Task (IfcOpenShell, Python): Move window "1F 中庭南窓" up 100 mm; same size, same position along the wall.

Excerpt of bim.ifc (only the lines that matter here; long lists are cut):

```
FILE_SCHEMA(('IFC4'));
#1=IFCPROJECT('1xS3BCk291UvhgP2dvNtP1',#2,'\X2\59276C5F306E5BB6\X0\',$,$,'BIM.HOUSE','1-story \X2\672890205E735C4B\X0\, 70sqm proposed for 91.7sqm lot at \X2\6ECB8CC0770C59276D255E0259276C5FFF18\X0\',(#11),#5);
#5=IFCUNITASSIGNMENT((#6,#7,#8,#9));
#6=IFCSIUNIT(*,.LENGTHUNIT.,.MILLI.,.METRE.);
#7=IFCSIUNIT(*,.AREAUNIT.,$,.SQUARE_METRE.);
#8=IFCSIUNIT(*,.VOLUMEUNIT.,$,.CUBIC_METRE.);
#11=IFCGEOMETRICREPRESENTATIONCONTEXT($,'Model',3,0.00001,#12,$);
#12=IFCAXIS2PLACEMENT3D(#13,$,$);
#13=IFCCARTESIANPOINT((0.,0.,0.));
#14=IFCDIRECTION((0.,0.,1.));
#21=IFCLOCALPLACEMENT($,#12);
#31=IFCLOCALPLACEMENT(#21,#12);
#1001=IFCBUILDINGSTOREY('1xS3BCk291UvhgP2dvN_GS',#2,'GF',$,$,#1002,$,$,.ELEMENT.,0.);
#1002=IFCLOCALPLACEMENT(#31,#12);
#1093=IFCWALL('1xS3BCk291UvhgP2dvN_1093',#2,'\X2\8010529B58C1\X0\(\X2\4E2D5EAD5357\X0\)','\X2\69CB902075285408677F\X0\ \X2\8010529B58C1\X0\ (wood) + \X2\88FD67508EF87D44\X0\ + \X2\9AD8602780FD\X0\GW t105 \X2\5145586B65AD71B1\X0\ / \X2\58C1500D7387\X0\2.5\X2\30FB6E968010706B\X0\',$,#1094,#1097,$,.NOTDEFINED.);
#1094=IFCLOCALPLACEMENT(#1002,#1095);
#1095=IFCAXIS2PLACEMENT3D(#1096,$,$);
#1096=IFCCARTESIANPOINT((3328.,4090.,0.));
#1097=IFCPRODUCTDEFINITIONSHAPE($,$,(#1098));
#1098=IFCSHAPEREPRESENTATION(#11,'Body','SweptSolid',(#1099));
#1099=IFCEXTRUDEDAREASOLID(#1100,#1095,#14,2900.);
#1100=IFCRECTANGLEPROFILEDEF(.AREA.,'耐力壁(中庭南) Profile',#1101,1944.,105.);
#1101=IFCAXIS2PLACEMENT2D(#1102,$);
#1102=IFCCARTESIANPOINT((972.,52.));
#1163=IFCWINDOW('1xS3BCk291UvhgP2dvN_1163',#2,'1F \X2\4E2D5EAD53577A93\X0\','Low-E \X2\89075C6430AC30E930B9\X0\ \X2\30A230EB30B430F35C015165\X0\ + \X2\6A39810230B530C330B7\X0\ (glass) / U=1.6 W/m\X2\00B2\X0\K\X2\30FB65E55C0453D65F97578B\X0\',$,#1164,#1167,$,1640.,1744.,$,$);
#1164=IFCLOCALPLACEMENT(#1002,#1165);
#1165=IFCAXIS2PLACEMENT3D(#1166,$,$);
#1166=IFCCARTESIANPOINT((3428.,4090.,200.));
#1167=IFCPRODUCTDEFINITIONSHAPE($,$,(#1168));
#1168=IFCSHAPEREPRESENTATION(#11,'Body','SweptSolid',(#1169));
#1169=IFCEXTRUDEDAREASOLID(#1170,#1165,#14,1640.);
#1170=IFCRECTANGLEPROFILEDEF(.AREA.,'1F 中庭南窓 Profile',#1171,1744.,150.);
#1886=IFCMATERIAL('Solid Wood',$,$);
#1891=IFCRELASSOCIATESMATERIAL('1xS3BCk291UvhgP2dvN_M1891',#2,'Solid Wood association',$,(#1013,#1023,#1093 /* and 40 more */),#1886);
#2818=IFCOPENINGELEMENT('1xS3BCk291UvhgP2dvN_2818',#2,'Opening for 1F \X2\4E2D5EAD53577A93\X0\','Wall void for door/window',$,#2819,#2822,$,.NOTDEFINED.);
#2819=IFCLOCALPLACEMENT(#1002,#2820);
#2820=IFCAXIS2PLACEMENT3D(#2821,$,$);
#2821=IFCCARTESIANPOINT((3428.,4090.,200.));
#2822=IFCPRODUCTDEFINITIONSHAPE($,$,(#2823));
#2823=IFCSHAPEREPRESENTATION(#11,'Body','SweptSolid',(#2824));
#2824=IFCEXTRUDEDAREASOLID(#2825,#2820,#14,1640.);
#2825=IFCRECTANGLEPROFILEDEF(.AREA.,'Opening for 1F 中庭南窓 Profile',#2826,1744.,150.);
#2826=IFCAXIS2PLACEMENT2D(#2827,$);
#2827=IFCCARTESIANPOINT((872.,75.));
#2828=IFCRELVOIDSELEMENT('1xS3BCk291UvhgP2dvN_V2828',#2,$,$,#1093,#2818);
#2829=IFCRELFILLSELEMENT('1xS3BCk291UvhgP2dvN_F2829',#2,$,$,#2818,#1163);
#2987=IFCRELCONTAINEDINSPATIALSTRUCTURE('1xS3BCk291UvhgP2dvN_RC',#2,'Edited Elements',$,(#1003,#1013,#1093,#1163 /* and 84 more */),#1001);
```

```python
import numpy as np
import ifcopenshell
import ifcopenshell.api.geometry
import ifcopenshell.util.placement
import ifcopenshell.util.unit

model = ifcopenshell.open("bim.ifc")
unit_scale = ifcopenshell.util.unit.calculate_unit_scale(model)

window = model.by_guid("1xS3BCk291UvhgP2dvN_1163")
opening = window.FillsVoids[0].RelatingOpeningElement
dz = 0.1 / unit_scale

shift = np.array([0.0, 0.0, dz])
# The window is not placed relative to its opening, so move both.
for product in (opening, window):
    matrix = ifcopenshell.util.placement.get_local_placement(product.ObjectPlacement)
    matrix[:3, 3] += shift
    ifcopenshell.api.geometry.edit_object_placement(model, product=product, matrix=matrix, is_si=False)

print(f"moved by {dz * unit_scale:+.3f} m")

model.write("bim_updated.ifc")
```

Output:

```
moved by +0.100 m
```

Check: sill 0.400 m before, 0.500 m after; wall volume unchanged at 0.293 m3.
